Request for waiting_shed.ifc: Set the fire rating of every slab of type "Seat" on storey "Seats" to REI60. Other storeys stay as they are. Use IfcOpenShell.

First a look at what the model holds.

```python
import ifcopenshell
import ifcopenshell.util.element

model = ifcopenshell.open("waiting_shed.ifc")
print(model.schema)
storey = next(s for s in model.by_type("IfcBuildingStorey") if s.Name == "Seats")
slabs = [e for e in ifcopenshell.util.element.get_decomposition(storey) if e.is_a("IfcSlab")]
seen = {}
for e in slabs:
    element_type = ifcopenshell.util.element.get_type(e)
    key = (element_type.Name if element_type != e and element_type else None, ifcopenshell.util.element.get_pset(e, "Pset_SlabCommon", "FireRating"))
    seen[key] = seen.get(key, 0) + 1
for (name, value), count in sorted(seen.items(), key=str):
    print(count, "x", name, "|", value)
```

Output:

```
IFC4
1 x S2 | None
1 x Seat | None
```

```python
import ifcopenshell
import ifcopenshell.api.pset
import ifcopenshell.util.element

model = ifcopenshell.open("waiting_shed.ifc")

storey = next(s for s in model.by_type("IfcBuildingStorey") if s.Name == "Seats")
slabs = [e for e in ifcopenshell.util.element.get_decomposition(storey) if e.is_a("IfcSlab")]

count = 0
for e in slabs:
    element_type = ifcopenshell.util.element.get_type(e)
    if element_type in (None, e) or element_type.Name != "Seat":
        continue
    # add_pset returns the element's existing set when there is one.
    pset = ifcopenshell.api.pset.add_pset(model, product=e, name="Pset_SlabCommon")
    ifcopenshell.api.pset.edit_pset(model, pset=pset, properties={"FireRating": "REI60"})
    count += 1

print(count, "slabs updated")

model.write("waiting_shed_v2.ifc")
```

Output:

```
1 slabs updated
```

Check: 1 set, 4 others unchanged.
